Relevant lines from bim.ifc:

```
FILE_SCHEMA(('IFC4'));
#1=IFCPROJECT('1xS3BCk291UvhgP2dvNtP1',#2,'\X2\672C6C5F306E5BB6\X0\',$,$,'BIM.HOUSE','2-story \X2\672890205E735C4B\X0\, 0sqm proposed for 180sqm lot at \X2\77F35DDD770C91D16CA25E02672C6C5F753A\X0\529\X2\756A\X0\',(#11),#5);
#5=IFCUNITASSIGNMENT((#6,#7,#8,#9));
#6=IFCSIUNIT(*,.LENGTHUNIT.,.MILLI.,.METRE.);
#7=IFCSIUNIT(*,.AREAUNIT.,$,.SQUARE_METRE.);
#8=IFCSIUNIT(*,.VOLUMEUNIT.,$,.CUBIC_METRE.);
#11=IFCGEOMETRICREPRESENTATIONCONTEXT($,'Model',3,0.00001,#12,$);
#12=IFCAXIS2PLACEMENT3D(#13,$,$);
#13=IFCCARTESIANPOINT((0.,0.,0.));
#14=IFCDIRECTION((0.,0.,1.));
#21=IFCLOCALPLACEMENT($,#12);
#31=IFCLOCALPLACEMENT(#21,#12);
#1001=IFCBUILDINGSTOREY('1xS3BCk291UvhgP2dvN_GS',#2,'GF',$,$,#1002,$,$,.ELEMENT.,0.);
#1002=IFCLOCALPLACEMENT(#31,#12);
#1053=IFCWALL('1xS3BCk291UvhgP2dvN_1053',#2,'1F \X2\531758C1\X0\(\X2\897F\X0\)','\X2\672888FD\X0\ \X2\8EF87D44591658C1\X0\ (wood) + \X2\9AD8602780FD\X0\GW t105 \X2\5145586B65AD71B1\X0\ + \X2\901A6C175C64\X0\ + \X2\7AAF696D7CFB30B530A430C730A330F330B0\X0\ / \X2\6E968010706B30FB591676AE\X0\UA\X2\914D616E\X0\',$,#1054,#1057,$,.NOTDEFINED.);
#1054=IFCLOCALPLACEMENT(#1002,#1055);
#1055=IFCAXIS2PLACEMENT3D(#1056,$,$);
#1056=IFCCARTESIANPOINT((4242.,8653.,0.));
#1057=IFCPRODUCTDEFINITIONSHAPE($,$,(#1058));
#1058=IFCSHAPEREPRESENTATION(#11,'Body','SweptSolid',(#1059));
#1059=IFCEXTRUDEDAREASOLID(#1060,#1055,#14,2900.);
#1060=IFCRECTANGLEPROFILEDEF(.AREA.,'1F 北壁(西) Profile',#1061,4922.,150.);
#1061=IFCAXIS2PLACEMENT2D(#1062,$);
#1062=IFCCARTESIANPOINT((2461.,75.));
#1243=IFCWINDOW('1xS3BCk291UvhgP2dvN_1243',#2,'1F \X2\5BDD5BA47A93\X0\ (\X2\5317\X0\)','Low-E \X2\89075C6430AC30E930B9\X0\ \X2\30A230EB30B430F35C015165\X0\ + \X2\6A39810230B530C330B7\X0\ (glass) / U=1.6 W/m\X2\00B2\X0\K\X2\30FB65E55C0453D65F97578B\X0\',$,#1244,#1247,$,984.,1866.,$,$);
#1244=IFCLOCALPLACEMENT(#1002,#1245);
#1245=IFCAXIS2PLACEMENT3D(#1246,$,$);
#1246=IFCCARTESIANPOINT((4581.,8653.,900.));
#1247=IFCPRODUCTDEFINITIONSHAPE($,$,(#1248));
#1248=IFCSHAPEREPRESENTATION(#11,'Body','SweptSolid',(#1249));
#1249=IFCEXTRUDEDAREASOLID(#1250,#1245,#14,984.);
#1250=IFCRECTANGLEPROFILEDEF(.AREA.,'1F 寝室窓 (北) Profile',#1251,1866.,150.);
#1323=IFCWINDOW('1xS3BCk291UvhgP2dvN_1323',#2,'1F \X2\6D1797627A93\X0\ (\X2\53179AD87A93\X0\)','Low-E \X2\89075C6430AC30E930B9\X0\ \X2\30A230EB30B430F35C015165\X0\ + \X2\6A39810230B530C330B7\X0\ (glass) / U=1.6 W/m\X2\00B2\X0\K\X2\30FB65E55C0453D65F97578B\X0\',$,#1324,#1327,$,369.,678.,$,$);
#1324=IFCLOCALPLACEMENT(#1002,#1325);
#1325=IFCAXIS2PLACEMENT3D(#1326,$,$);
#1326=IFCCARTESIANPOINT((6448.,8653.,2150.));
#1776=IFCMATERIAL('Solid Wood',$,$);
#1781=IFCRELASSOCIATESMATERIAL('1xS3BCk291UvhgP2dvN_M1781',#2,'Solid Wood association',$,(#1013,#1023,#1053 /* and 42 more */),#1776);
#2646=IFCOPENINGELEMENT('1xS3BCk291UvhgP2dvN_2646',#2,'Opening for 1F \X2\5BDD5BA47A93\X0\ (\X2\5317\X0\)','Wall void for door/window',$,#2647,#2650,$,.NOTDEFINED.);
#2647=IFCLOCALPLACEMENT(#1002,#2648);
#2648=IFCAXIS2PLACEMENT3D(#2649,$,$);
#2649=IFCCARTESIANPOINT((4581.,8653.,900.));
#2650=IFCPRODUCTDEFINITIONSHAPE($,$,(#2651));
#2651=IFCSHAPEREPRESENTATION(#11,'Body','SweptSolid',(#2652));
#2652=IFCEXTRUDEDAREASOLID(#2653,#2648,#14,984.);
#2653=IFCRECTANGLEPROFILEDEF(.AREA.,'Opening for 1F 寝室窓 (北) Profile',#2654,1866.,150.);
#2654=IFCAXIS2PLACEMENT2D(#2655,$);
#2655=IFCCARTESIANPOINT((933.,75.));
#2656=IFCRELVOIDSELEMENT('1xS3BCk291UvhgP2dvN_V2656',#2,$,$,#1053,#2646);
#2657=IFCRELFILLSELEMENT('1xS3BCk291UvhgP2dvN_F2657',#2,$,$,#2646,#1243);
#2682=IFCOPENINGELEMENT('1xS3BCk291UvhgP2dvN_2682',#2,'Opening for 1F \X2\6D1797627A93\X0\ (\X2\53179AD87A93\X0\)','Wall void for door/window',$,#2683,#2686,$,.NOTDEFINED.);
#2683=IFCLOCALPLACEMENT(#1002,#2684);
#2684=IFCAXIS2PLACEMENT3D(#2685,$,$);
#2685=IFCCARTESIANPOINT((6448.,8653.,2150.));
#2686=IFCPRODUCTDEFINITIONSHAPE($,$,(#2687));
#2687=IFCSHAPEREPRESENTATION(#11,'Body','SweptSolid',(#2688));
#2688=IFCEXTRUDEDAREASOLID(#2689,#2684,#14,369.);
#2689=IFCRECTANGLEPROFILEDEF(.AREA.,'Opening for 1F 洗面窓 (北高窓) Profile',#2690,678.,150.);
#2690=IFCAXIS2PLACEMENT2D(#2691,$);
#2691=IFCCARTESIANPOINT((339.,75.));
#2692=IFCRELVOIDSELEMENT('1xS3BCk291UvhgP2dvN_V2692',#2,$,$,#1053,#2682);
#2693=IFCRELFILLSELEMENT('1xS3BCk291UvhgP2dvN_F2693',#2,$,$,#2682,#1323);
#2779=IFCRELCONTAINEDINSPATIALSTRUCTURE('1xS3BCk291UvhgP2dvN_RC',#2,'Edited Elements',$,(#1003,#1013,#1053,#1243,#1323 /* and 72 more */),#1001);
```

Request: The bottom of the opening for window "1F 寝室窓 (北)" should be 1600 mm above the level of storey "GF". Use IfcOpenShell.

```python
import numpy as np
import ifcopenshell
import ifcopenshell.api.geometry
import ifcopenshell.geom
import ifcopenshell.util.element
import ifcopenshell.util.placement
import ifcopenshell.util.shape
import ifcopenshell.util.unit

model = ifcopenshell.open("bim.ifc")
unit_scale = ifcopenshell.util.unit.calculate_unit_scale(model)

window = model.by_guid("1xS3BCk291UvhgP2dvN_1243")
opening = window.FillsVoids[0].RelatingOpeningElement
storey = ifcopenshell.util.element.get_container(window, ifc_class="IfcBuildingStorey")
level = ifcopenshell.util.placement.get_local_placement(storey.ObjectPlacement)[2, 3]

# The opening's origin need not be at the sill, so measure its lowest point.
shape = ifcopenshell.geom.create_shape(ifcopenshell.geom.settings(), opening)
bottom = ifcopenshell.util.shape.get_shape_bottom_elevation(shape, shape.geometry) / unit_scale
dz = level + 1.6 / unit_scale - bottom

shift = np.array([0.0, 0.0, dz])
# The window is not placed relative to its opening, so move both.
for product in (opening, window):
    matrix = ifcopenshell.util.placement.get_local_placement(product.ObjectPlacement)
    matrix[:3, 3] += shift
    ifcopenshell.api.geometry.edit_object_placement(model, product=product, matrix=matrix, is_si=False)

print(f"moved by {dz * unit_scale:+.3f} m")

model.write("bim_v2.ifc")
```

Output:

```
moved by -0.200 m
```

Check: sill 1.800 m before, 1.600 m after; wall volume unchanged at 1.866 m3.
